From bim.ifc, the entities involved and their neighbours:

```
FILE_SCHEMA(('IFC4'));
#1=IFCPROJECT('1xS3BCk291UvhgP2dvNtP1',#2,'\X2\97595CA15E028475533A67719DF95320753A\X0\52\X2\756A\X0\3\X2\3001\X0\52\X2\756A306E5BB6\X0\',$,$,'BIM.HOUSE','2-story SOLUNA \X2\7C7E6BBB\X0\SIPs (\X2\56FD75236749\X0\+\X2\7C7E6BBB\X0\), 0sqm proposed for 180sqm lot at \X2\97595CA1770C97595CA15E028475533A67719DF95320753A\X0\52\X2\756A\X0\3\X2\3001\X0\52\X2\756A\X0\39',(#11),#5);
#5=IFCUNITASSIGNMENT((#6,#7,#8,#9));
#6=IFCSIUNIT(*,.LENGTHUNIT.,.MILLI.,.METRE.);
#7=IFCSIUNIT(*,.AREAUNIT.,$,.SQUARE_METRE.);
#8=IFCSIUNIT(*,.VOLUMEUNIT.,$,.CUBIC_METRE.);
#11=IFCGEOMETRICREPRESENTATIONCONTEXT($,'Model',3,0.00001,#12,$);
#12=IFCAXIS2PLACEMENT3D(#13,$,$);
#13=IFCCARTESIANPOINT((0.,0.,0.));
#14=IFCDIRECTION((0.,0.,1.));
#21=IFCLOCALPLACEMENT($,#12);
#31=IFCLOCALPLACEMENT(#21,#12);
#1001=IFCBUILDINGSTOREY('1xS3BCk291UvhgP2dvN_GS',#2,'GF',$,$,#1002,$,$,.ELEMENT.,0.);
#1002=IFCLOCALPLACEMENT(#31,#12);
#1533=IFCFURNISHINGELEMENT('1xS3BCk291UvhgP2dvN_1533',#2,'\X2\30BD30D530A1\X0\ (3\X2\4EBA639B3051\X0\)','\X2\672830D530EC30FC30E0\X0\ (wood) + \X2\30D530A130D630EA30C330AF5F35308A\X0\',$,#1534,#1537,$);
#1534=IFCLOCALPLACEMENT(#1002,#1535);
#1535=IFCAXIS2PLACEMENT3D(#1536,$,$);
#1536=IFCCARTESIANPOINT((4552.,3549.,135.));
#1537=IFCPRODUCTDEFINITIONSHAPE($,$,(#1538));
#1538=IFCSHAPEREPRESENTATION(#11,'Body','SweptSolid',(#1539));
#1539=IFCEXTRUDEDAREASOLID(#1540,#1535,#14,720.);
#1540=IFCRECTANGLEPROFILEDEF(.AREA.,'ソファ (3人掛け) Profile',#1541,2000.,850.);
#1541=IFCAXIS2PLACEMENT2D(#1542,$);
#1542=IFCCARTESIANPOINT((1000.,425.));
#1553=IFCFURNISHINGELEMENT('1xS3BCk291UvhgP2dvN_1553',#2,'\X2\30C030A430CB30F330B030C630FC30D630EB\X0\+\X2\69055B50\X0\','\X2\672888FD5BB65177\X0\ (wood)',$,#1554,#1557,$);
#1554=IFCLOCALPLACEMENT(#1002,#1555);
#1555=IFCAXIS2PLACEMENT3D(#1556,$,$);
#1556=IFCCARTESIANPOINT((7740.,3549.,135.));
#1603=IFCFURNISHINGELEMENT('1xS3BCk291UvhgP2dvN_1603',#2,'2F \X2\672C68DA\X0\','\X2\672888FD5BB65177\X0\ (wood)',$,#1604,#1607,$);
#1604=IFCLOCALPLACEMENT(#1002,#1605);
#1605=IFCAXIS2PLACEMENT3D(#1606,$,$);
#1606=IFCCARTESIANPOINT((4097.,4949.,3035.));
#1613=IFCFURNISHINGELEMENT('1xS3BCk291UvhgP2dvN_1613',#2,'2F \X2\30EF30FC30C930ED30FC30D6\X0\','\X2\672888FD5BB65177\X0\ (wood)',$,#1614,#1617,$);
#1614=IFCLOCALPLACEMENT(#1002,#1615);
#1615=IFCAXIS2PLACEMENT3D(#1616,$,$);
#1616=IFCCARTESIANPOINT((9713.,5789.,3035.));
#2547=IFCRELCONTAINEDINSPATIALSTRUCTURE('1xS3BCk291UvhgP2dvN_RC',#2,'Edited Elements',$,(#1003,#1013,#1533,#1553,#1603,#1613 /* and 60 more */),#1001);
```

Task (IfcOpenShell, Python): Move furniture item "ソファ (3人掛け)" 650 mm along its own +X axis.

```python
import ifcopenshell
import ifcopenshell.api.geometry
import ifcopenshell.util.placement

model = ifcopenshell.open("bim.ifc")

item = model.by_guid("1xS3BCk291UvhgP2dvN_1533")
matrix = ifcopenshell.util.placement.get_local_placement(item.ObjectPlacement)
matrix[:3, 3] += matrix[:3, 0] * 650.0
ifcopenshell.api.geometry.edit_object_placement(model, product=item, matrix=matrix, is_si=False)

print(ifcopenshell.util.placement.get_local_placement(item.ObjectPlacement).round(3) + 0.0)

model.write("bim_rev.ifc")
```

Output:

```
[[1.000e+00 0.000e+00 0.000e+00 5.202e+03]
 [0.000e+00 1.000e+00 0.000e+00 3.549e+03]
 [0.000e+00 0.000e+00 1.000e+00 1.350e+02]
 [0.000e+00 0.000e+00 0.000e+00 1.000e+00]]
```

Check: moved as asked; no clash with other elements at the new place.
